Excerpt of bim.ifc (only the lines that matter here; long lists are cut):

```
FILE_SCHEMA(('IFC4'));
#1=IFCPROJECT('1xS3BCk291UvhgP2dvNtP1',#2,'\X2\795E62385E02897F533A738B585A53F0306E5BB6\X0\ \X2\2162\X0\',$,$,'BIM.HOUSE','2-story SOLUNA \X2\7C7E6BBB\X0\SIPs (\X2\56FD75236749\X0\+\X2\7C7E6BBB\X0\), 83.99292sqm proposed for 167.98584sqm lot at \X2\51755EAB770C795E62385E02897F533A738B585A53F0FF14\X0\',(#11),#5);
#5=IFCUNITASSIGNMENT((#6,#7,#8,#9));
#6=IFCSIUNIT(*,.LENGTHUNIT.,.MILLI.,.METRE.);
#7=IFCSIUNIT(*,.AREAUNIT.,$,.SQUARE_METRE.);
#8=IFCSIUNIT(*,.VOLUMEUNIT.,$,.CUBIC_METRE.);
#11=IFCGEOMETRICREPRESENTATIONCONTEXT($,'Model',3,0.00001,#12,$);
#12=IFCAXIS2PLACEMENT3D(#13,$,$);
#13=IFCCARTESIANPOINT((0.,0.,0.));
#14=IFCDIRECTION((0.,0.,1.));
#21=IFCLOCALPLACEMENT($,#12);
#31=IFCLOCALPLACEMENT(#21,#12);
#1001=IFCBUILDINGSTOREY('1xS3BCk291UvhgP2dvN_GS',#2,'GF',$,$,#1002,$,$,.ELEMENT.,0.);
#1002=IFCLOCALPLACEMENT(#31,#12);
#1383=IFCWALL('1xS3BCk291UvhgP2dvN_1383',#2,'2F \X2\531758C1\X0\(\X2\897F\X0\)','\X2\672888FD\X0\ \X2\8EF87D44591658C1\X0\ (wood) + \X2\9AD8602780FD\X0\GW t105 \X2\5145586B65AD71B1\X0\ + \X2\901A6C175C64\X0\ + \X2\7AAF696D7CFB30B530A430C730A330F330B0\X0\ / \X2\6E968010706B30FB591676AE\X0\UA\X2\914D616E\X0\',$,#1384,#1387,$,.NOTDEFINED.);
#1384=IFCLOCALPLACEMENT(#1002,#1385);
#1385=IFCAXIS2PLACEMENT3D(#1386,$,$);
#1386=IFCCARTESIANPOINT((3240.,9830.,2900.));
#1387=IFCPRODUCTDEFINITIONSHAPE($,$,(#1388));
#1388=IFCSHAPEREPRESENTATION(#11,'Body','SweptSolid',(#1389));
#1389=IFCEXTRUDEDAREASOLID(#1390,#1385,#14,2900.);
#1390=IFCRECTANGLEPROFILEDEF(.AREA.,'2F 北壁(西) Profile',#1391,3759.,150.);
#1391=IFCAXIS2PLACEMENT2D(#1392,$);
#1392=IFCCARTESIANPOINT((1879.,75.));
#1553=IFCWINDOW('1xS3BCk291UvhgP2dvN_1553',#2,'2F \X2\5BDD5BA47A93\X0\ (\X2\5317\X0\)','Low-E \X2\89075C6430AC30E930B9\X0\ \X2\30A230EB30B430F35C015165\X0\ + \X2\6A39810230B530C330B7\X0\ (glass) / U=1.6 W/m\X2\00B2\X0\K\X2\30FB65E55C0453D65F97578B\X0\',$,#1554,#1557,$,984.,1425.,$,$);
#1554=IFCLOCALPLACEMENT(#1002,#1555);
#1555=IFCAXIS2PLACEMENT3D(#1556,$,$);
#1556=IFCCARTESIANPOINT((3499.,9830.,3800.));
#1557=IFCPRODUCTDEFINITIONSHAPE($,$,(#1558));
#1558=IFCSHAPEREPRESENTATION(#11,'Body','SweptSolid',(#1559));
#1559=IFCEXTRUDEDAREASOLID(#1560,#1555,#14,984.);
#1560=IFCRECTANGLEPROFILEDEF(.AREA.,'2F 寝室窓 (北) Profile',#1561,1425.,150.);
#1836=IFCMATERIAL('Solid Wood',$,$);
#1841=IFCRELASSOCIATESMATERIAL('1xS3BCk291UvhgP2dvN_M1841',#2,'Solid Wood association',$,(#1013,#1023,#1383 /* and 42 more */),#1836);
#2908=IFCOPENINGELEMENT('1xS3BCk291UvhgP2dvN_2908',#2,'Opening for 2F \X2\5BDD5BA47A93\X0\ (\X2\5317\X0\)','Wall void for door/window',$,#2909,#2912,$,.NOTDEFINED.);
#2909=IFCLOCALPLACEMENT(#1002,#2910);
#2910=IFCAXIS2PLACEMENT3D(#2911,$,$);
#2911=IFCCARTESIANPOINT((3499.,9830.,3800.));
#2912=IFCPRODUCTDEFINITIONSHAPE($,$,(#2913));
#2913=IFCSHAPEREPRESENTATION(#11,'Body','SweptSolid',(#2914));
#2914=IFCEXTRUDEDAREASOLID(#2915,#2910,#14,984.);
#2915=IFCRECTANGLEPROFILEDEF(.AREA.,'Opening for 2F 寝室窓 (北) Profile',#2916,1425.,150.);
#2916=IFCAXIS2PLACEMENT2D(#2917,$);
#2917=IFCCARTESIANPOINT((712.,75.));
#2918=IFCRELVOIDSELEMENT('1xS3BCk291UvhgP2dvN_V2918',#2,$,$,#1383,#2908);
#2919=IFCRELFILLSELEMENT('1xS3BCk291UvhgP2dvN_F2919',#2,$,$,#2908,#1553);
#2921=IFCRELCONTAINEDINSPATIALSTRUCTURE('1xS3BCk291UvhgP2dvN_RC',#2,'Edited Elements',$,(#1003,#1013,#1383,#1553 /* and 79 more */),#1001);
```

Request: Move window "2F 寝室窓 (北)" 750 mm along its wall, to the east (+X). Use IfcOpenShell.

```python
import ifcopenshell
import ifcopenshell.api.geometry
import ifcopenshell.util.placement
import ifcopenshell.util.unit

model = ifcopenshell.open("bim.ifc")
unit_scale = ifcopenshell.util.unit.calculate_unit_scale(model)

window = model.by_id(1553)
opening = window.FillsVoids[0].RelatingOpeningElement
wall = opening.VoidsElements[0].RelatingBuildingElement

wall_matrix = ifcopenshell.util.placement.get_local_placement(wall.ObjectPlacement)
shift = wall_matrix[:3, 0] * 0.75 / unit_scale
before = ifcopenshell.util.placement.get_local_placement(window.ObjectPlacement)[:3, 3].copy()

# The window is not placed relative to its opening, so move both.
for product in (opening, window):
    matrix = ifcopenshell.util.placement.get_local_placement(product.ObjectPlacement)
    matrix[:3, 3] += shift
    ifcopenshell.api.geometry.edit_object_placement(model, product=product, matrix=matrix, is_si=False)

after = ifcopenshell.util.placement.get_local_placement(window.ObjectPlacement)[:3, 3]
print("window moved by", (after - before).round(3) + 0.0)

model.write("bim_updated.ifc")
```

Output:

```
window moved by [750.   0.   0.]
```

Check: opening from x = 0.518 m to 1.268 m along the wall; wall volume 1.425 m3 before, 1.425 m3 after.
